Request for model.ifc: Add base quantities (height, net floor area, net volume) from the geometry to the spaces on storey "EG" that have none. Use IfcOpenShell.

First a look at what the model holds.

```python
import ifcopenshell
import ifcopenshell.util.element
import ifcopenshell.util.unit

model = ifcopenshell.open("model.ifc")
print(model.schema)
for unit_type in ("LENGTHUNIT", "AREAUNIT", "VOLUMEUNIT"):
    print(unit_type, ifcopenshell.util.unit.calculate_unit_scale(model, unit_type))
storey = next(s for s in model.by_type("IfcBuildingStorey") if s.Name == "EG")
spaces = [e for e in ifcopenshell.util.element.get_decomposition(storey) if e.is_a("IfcSpace")]
for e in sorted(spaces, key=lambda e: e.id()):
    print(e.id(), e.is_a(), e.Name, list(ifcopenshell.util.element.get_psets(e, qtos_only=True)), sep=" | ")
```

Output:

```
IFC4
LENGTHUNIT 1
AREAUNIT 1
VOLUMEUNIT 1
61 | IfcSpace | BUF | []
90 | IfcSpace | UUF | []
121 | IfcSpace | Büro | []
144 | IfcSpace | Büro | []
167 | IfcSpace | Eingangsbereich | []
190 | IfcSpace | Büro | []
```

```python
import ifcopenshell
import ifcopenshell.api.pset
import ifcopenshell.geom
import ifcopenshell.util.element
import ifcopenshell.util.shape
import ifcopenshell.util.unit

model = ifcopenshell.open("model.ifc")
unit_scale = ifcopenshell.util.unit.calculate_unit_scale(model)
area_scale = ifcopenshell.util.unit.calculate_unit_scale(model, "AREAUNIT")
volume_scale = ifcopenshell.util.unit.calculate_unit_scale(model, "VOLUMEUNIT")
settings = ifcopenshell.geom.settings()

storey = next(s for s in model.by_type("IfcBuildingStorey") if s.Name == "EG")
spaces = [e for e in ifcopenshell.util.element.get_decomposition(storey) if e.is_a("IfcSpace")]

for e in sorted(spaces, key=lambda e: e.id()):
    if ifcopenshell.util.element.get_psets(e, qtos_only=True, should_inherit=False):
        continue
    # Geometry comes back in metres, in the element's own axes.
    shape = ifcopenshell.geom.create_shape(settings, e)
    values = {
        "Height": ifcopenshell.util.shape.get_z(shape.geometry) / unit_scale,
        "NetFloorArea": ifcopenshell.util.shape.get_footprint_area(shape.geometry) / area_scale,
        "NetVolume": ifcopenshell.util.shape.get_volume(shape.geometry) / volume_scale,
    }
    qto = ifcopenshell.api.pset.add_qto(model, product=e, name="Qto_SpaceBaseQuantities")
    ifcopenshell.api.pset.edit_qto(model, qto=qto, properties=values)
    print(e.id(), {k: round(v, 3) for k, v in values.items()})

model.write("model_edited.ifc")
```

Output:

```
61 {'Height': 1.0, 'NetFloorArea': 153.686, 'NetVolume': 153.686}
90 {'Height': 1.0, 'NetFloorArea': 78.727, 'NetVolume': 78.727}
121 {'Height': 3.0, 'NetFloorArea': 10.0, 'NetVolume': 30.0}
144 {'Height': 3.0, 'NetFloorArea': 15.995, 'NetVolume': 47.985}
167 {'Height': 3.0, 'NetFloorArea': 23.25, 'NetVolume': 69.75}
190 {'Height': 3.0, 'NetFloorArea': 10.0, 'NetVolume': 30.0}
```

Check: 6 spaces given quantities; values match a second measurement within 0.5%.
